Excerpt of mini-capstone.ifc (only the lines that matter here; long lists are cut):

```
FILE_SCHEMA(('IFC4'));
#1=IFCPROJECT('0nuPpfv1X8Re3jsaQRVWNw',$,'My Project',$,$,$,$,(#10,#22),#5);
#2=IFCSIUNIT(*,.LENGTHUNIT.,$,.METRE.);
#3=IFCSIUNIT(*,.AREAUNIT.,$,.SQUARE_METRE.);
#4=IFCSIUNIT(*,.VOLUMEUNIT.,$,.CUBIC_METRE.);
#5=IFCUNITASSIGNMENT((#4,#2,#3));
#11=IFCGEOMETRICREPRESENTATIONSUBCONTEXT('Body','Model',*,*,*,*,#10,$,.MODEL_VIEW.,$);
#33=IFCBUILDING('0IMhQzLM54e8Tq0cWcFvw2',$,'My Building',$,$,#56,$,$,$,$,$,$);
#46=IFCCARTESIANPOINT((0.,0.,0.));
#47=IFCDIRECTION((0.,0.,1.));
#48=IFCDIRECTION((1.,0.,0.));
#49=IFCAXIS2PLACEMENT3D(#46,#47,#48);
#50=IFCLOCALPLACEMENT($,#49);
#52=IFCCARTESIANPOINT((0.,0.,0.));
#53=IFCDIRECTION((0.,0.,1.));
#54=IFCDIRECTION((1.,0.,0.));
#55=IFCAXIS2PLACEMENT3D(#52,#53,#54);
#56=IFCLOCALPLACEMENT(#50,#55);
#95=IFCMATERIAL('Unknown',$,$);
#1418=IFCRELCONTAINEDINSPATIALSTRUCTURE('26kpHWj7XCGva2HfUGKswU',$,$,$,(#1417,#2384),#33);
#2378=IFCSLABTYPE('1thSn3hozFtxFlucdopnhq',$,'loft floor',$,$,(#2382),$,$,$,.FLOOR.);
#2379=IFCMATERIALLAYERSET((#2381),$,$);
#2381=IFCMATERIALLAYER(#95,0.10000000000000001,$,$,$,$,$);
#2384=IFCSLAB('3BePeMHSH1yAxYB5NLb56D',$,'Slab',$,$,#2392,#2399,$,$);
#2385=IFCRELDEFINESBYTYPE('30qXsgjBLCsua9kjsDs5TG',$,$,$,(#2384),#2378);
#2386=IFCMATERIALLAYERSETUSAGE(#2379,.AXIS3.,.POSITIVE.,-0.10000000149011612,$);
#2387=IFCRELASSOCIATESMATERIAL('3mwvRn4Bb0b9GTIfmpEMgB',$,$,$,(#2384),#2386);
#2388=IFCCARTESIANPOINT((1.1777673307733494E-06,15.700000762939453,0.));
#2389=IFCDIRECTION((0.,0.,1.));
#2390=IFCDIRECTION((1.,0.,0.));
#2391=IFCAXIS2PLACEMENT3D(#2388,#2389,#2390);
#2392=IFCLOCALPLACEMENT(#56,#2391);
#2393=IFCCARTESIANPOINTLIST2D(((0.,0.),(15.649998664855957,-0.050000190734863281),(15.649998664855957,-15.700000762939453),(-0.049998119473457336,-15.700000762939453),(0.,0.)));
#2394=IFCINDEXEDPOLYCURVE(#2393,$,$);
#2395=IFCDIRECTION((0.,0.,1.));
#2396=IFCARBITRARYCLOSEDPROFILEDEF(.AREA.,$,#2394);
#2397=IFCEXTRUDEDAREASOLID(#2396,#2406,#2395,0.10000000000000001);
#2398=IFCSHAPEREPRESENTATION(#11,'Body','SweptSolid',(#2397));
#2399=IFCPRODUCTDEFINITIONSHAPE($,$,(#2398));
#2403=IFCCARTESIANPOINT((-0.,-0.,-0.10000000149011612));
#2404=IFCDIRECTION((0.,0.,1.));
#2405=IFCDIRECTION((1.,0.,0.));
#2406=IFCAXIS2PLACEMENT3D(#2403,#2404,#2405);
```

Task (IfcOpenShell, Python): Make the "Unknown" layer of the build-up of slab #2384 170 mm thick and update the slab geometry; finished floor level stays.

```python
import ifcopenshell
import ifcopenshell.util.element
import ifcopenshell.util.representation
import ifcopenshell.util.unit

model = ifcopenshell.open("mini-capstone.ifc")
unit_scale = ifcopenshell.util.unit.calculate_unit_scale(model)

layer_set = model.by_id(2379)
layer = next(l for l in layer_set.MaterialLayers if l.Material and l.Material.Name == "Unknown")
change = 0.17 / unit_scale - layer.LayerThickness
layer.LayerThickness += change

# Geometry does not follow the layer set by itself.
slabs = [e for e in ifcopenshell.util.element.get_elements_by_material(model, layer_set) if e.is_a("IfcSlab")]
for slab in sorted(slabs, key=lambda e: e.id()):
    body = ifcopenshell.util.representation.get_representation(slab, "Model", "Body")
    solid = body.Items[0]
    old_depth = solid.Depth
    solid.Depth += change
    # Extruded upwards: lower the start of the extrusion so the top stays.
    x, y, z = solid.Position.Location.Coordinates
    solid.Position.Location = model.createIfcCartesianPoint((x, y, z - change))
    print(slab.id(), f"{old_depth:g} -> {solid.Depth:g}")

# The layers are counted up from the underside, which has moved.
for usage in {ifcopenshell.util.element.get_material(slab) for slab in slabs}:
    usage.OffsetFromReferenceLine -= change

model.write("mini-capstone_updated.ifc")
```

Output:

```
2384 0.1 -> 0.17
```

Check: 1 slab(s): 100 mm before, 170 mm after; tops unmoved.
